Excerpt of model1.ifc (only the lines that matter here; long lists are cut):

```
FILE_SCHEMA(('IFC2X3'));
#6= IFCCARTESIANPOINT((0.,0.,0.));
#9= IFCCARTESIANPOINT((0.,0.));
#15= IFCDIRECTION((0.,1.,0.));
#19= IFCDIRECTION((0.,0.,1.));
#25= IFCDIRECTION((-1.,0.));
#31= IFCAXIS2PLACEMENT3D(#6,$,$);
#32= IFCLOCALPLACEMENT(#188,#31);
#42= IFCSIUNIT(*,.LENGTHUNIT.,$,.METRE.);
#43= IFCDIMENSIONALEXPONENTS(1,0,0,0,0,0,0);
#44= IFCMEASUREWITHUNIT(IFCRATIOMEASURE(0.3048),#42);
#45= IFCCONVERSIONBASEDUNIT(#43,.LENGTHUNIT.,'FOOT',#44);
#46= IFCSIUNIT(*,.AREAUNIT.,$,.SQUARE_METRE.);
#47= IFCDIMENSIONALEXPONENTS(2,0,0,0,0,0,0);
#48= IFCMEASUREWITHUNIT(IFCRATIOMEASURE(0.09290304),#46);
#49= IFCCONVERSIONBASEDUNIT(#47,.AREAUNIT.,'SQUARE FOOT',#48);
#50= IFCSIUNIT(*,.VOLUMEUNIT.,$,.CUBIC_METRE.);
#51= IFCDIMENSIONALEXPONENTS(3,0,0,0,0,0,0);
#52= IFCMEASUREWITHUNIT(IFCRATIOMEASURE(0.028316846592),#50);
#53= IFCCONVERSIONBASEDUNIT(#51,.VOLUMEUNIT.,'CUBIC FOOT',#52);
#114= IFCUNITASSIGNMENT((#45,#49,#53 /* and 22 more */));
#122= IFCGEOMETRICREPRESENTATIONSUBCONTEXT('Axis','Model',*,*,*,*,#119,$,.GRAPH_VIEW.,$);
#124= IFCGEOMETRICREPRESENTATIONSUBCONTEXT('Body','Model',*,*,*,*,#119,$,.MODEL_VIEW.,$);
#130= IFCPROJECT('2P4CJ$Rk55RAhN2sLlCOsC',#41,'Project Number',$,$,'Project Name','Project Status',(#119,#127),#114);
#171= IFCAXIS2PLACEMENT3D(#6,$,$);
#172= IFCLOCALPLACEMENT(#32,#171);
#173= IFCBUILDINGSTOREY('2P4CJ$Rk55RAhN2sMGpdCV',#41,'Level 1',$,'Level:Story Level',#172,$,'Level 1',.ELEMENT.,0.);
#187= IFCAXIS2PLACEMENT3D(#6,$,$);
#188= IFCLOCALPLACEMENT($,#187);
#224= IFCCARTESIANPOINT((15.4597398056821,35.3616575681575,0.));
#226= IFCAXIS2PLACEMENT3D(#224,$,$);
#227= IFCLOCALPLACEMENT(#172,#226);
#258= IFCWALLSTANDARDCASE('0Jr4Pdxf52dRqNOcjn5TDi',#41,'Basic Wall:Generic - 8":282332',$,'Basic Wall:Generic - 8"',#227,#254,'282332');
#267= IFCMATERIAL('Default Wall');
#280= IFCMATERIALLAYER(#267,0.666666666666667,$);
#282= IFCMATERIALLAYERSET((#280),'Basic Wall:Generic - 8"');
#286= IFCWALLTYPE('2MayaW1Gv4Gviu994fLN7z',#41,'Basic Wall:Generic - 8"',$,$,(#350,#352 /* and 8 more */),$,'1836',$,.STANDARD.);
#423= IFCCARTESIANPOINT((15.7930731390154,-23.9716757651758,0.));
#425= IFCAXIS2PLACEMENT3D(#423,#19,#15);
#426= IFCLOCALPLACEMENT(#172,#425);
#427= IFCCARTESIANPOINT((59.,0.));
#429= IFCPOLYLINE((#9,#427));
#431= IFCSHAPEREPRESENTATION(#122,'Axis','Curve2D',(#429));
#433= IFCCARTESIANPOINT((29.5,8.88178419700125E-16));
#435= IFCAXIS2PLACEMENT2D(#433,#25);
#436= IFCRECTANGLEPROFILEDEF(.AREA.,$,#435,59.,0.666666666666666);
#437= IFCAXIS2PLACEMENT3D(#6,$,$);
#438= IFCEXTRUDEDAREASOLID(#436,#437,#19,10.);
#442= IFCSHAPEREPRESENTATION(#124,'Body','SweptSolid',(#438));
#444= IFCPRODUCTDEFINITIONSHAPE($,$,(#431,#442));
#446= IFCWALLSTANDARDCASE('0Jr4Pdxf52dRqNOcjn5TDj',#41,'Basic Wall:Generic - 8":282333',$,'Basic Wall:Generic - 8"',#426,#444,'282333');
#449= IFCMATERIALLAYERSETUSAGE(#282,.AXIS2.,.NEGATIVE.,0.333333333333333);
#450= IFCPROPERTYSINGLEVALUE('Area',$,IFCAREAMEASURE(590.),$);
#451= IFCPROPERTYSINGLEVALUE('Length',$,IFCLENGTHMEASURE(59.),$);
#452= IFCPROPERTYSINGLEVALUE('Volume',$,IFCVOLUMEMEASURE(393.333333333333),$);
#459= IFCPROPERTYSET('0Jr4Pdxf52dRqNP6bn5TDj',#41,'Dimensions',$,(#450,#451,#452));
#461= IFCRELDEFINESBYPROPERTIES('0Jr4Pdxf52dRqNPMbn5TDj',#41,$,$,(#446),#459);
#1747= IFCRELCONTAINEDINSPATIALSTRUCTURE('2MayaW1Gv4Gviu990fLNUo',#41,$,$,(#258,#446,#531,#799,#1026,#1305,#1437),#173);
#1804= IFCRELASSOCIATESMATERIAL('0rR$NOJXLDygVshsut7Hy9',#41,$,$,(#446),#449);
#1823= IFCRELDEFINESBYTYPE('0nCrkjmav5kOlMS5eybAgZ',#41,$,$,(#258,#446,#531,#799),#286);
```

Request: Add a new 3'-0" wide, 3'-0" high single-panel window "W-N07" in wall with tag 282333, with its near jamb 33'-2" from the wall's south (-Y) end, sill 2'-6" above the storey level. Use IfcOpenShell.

```python
import numpy as np
import ifcopenshell
import ifcopenshell.api.feature
import ifcopenshell.api.geometry
import ifcopenshell.api.pset
import ifcopenshell.api.root
import ifcopenshell.api.spatial
import ifcopenshell.api.type
import ifcopenshell.geom
import ifcopenshell.util.element
import ifcopenshell.util.placement
import ifcopenshell.util.representation
import ifcopenshell.util.shape
import ifcopenshell.util.unit

model = ifcopenshell.open("model1.ifc")
unit_scale = ifcopenshell.util.unit.calculate_unit_scale(model)
area_scale = ifcopenshell.util.unit.calculate_unit_scale(model, "AREAUNIT")
volume_scale = ifcopenshell.util.unit.calculate_unit_scale(model, "VOLUMEUNIT")
settings = ifcopenshell.geom.settings()


def volume(element):
    """Net volume in cubic metres, openings subtracted."""
    shape = ifcopenshell.geom.create_shape(settings, element)
    return ifcopenshell.util.shape.get_volume(shape.geometry)


wall = model.by_guid("0Jr4Pdxf52dRqNOcjn5TDj")
storey = ifcopenshell.util.element.get_container(wall, ifc_class="IfcBuildingStorey")
context = ifcopenshell.util.representation.get_context(model, "Model", "Body", "MODEL_VIEW")
before = volume(wall)

width, height, from_end, sill = 0.9144, 0.9144, 10.1092, 0.762  # metres

# The wall runs along its own X axis, and the end named is its -X end.
wall_shape = ifcopenshell.geom.create_shape(settings, wall)
x, y, z = ifcopenshell.util.shape.get_vertices(wall_shape.geometry).T
start = x.min() + from_end
face, thickness = float(y.min()), float(y.max() - y.min())
wall_matrix = ifcopenshell.util.placement.get_local_placement(wall.ObjectPlacement)
level = ifcopenshell.util.placement.get_local_placement(storey.ObjectPlacement)[2, 3]


def in_wall(x, y):
    """Placement at x, y metres in the wall's axes, at sill height."""
    matrix = wall_matrix.copy()
    matrix[:, 3] = wall_matrix @ np.array([x / unit_scale, y / unit_scale, 0.0, 1.0])
    matrix[2, 3] = level + sill / unit_scale
    return matrix


# Opening: a box that overshoots both wall faces by 50 mm.
opening = ifcopenshell.api.root.create_entity(model, ifc_class="IfcOpeningElement")
box = ifcopenshell.api.geometry.add_wall_representation(
    model, context=context, length=width, height=height, thickness=thickness + 0.1
)
ifcopenshell.api.geometry.assign_representation(model, product=opening, representation=box)
ifcopenshell.api.geometry.edit_object_placement(model, product=opening, matrix=in_wall(start, face - 0.05), is_si=False)
ifcopenshell.api.feature.add_feature(model, feature=opening, element=wall)

window = ifcopenshell.api.root.create_entity(model, ifc_class="IfcWindow", name="W-N07")
window.OverallWidth, window.OverallHeight = width / unit_scale, height / unit_scale
body = ifcopenshell.api.geometry.add_window_representation(
    model,
    context=context,
    overall_width=window.OverallWidth,
    overall_height=window.OverallHeight,
    partition_type="SINGLE_PANEL",
)
ifcopenshell.api.geometry.assign_representation(model, product=window, representation=body)
ifcopenshell.api.spatial.assign_container(model, products=[window], relating_structure=storey)
fills = ifcopenshell.api.feature.add_filling(model, opening=opening, element=window)
fills.OwnerHistory = window.OwnerHistory  # required in IFC2X3

# IFC2X3 keeps the operation on the window style.
style = ifcopenshell.api.root.create_entity(model, ifc_class="IfcWindowStyle", name="W-N07")
style.OperationType, style.ConstructionType = "SINGLE_PANEL", "NOTDEFINED"
style.ParameterTakesPrecedence = style.Sizeable = False
ifcopenshell.api.type.assign_type(model, related_objects=[window], relating_type=style)

# Centre the window in the wall's thickness.
ifcopenshell.api.geometry.edit_object_placement(model, product=window, matrix=in_wall(start, face), is_si=False)
window_shape = ifcopenshell.geom.create_shape(settings, window)
depth = ifcopenshell.util.shape.get_vertices(window_shape.geometry)[:, 1]
offset = face + thickness / 2 - (depth.min() + depth.max()) / 2
ifcopenshell.api.geometry.edit_object_placement(model, product=window, matrix=in_wall(start, offset), is_si=False)

after = volume(wall)

# Update the wall's stored quantities.
pset = model.by_id(ifcopenshell.util.element.get_pset(wall, "Dimensions", should_inherit=False)["id"])
ifcopenshell.api.pset.edit_pset(model, pset=pset, properties={
    "Area": model.create_entity("IfcAreaMeasure", after / thickness / area_scale),
    "Volume": model.create_entity("IfcVolumeMeasure", after / volume_scale),
})

print(f"wall volume {before:.3f} -> {after:.3f} m3")

model.write("model1-out.ifc")
```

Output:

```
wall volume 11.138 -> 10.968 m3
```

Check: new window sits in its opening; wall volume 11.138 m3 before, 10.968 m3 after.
